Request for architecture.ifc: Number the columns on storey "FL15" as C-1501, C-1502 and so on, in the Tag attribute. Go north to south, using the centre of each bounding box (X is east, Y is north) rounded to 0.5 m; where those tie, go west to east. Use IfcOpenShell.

First a look at what the model holds.

```python
import ifcopenshell
import ifcopenshell.util.element
import ifcopenshell.util.placement

model = ifcopenshell.open("architecture.ifc")
print(model.schema)
storey = next(s for s in model.by_type("IfcBuildingStorey") if s.Name == "FL15")
columns = [e for e in ifcopenshell.util.element.get_decomposition(storey) if e.is_a("IfcColumn")]
for e in sorted(columns, key=lambda e: e.id()):
    origin = ifcopenshell.util.placement.get_local_placement(e.ObjectPlacement)[:3, 3]
    print(e.id(), e.Tag, e.Name, origin.round(2) + 0.0, sep=" | ")
```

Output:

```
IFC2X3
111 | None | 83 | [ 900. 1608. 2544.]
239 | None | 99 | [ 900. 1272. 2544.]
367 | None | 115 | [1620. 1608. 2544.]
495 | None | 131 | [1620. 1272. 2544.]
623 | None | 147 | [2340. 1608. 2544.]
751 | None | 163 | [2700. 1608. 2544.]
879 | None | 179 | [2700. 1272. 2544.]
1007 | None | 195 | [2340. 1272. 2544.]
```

```python
import ifcopenshell
import ifcopenshell.geom
import ifcopenshell.util.element
import ifcopenshell.util.shape

model = ifcopenshell.open("architecture.ifc")
settings = ifcopenshell.geom.settings()
settings.set("use-world-coords", True)


def centre(element):
    shape = ifcopenshell.geom.create_shape(settings, element)
    return ifcopenshell.util.shape.get_bbox_centroid(shape.geometry)


storey = next(s for s in model.by_type("IfcBuildingStorey") if s.Name == "FL15")
columns = [e for e in ifcopenshell.util.element.get_decomposition(storey) if e.is_a("IfcColumn")]

# Insertion points can sit at a corner or the storey origin, so sort by the geometry (in metres).
centres = {e: centre(e) for e in columns}
columns.sort(key=lambda e: (-round(centres[e][1] / 0.5), centres[e][0]))

for i, e in enumerate(columns, start=1):
    number = f"C-15{i:02d}"
    e.Tag = number
    print(e.id(), number)

model.write("architecture_updated.ifc")
```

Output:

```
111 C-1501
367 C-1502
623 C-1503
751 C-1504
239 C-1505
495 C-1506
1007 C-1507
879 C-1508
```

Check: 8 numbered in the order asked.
